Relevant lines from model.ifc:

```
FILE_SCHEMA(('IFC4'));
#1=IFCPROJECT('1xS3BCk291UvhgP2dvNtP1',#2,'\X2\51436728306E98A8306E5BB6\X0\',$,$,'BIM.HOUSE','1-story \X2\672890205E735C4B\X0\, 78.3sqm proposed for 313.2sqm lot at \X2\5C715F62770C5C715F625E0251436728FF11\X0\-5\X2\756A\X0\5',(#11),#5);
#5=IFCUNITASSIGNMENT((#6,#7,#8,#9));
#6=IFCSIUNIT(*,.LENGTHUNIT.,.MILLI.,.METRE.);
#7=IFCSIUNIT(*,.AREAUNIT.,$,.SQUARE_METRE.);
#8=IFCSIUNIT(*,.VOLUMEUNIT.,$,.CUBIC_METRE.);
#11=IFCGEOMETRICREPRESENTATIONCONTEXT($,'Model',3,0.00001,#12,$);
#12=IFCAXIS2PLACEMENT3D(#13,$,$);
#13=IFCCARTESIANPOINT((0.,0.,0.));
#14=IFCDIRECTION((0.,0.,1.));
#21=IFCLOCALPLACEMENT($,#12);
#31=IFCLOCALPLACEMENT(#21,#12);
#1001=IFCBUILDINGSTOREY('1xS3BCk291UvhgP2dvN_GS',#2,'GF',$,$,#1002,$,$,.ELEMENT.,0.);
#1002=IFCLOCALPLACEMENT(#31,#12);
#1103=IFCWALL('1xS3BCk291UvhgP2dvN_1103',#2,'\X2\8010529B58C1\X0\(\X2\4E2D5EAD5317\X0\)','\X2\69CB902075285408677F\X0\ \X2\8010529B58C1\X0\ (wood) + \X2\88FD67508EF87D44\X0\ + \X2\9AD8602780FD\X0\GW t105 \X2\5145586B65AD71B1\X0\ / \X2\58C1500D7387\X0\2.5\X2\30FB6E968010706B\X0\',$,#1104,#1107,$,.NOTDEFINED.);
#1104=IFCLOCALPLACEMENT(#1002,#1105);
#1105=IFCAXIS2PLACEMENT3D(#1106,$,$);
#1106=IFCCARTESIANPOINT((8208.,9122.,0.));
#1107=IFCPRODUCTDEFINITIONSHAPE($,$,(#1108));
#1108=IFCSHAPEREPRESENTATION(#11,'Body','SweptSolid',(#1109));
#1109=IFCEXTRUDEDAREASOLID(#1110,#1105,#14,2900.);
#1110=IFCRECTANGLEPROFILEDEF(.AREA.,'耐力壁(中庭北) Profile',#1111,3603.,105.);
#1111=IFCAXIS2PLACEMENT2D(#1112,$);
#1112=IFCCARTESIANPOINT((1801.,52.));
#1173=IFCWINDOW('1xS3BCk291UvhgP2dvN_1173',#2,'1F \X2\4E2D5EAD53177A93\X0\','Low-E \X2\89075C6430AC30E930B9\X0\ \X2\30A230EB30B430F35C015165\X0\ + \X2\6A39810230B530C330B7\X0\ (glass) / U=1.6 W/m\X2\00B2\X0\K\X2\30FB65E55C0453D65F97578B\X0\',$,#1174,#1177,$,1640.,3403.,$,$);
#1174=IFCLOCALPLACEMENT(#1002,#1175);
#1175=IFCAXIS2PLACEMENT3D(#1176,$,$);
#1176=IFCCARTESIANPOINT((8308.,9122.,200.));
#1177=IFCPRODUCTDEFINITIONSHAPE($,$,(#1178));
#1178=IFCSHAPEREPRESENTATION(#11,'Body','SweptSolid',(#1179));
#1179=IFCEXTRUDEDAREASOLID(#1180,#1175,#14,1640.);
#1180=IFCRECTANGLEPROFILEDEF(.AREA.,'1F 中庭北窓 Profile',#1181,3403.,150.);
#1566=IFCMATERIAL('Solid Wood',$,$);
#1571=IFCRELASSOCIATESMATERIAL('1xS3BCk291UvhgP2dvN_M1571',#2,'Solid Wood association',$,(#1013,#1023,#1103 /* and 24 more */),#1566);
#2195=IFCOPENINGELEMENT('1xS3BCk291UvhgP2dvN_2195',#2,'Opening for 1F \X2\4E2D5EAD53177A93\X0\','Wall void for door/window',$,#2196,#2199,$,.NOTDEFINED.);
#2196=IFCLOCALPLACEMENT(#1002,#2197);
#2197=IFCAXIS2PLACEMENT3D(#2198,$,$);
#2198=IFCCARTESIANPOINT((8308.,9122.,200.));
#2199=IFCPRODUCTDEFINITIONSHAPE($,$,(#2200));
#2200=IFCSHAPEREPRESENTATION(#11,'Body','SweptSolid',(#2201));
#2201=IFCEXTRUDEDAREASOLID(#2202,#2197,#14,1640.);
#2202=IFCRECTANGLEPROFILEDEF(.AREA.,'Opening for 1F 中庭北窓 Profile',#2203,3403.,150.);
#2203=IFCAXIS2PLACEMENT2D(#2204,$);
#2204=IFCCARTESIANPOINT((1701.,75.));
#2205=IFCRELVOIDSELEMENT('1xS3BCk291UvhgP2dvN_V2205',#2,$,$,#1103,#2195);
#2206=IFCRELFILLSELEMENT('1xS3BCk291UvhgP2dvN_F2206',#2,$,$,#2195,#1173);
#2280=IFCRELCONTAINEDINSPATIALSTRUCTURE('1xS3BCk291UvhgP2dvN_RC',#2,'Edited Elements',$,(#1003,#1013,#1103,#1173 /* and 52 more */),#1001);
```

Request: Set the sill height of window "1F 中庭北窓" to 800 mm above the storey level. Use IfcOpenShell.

```python
import numpy as np
import ifcopenshell
import ifcopenshell.api.geometry
import ifcopenshell.geom
import ifcopenshell.util.element
import ifcopenshell.util.placement
import ifcopenshell.util.shape
import ifcopenshell.util.unit

model = ifcopenshell.open("model.ifc")
unit_scale = ifcopenshell.util.unit.calculate_unit_scale(model)

window = model.by_id(1173)
opening = window.FillsVoids[0].RelatingOpeningElement
storey = ifcopenshell.util.element.get_container(window, ifc_class="IfcBuildingStorey")
level = ifcopenshell.util.placement.get_local_placement(storey.ObjectPlacement)[2, 3]

# The opening's origin need not be at the sill, so measure its lowest point.
shape = ifcopenshell.geom.create_shape(ifcopenshell.geom.settings(), opening)
bottom = ifcopenshell.util.shape.get_shape_bottom_elevation(shape, shape.geometry) / unit_scale
dz = level + 0.8 / unit_scale - bottom

shift = np.array([0.0, 0.0, dz])
# The window is not placed relative to its opening, so move both.
for product in (opening, window):
    matrix = ifcopenshell.util.placement.get_local_placement(product.ObjectPlacement)
    matrix[:3, 3] += shift
    ifcopenshell.api.geometry.edit_object_placement(model, product=product, matrix=matrix, is_si=False)

print(f"moved by {dz * unit_scale:+.3f} m")

model.write("model_v2.ifc")
```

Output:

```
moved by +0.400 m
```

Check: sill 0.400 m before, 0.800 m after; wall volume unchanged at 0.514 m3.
